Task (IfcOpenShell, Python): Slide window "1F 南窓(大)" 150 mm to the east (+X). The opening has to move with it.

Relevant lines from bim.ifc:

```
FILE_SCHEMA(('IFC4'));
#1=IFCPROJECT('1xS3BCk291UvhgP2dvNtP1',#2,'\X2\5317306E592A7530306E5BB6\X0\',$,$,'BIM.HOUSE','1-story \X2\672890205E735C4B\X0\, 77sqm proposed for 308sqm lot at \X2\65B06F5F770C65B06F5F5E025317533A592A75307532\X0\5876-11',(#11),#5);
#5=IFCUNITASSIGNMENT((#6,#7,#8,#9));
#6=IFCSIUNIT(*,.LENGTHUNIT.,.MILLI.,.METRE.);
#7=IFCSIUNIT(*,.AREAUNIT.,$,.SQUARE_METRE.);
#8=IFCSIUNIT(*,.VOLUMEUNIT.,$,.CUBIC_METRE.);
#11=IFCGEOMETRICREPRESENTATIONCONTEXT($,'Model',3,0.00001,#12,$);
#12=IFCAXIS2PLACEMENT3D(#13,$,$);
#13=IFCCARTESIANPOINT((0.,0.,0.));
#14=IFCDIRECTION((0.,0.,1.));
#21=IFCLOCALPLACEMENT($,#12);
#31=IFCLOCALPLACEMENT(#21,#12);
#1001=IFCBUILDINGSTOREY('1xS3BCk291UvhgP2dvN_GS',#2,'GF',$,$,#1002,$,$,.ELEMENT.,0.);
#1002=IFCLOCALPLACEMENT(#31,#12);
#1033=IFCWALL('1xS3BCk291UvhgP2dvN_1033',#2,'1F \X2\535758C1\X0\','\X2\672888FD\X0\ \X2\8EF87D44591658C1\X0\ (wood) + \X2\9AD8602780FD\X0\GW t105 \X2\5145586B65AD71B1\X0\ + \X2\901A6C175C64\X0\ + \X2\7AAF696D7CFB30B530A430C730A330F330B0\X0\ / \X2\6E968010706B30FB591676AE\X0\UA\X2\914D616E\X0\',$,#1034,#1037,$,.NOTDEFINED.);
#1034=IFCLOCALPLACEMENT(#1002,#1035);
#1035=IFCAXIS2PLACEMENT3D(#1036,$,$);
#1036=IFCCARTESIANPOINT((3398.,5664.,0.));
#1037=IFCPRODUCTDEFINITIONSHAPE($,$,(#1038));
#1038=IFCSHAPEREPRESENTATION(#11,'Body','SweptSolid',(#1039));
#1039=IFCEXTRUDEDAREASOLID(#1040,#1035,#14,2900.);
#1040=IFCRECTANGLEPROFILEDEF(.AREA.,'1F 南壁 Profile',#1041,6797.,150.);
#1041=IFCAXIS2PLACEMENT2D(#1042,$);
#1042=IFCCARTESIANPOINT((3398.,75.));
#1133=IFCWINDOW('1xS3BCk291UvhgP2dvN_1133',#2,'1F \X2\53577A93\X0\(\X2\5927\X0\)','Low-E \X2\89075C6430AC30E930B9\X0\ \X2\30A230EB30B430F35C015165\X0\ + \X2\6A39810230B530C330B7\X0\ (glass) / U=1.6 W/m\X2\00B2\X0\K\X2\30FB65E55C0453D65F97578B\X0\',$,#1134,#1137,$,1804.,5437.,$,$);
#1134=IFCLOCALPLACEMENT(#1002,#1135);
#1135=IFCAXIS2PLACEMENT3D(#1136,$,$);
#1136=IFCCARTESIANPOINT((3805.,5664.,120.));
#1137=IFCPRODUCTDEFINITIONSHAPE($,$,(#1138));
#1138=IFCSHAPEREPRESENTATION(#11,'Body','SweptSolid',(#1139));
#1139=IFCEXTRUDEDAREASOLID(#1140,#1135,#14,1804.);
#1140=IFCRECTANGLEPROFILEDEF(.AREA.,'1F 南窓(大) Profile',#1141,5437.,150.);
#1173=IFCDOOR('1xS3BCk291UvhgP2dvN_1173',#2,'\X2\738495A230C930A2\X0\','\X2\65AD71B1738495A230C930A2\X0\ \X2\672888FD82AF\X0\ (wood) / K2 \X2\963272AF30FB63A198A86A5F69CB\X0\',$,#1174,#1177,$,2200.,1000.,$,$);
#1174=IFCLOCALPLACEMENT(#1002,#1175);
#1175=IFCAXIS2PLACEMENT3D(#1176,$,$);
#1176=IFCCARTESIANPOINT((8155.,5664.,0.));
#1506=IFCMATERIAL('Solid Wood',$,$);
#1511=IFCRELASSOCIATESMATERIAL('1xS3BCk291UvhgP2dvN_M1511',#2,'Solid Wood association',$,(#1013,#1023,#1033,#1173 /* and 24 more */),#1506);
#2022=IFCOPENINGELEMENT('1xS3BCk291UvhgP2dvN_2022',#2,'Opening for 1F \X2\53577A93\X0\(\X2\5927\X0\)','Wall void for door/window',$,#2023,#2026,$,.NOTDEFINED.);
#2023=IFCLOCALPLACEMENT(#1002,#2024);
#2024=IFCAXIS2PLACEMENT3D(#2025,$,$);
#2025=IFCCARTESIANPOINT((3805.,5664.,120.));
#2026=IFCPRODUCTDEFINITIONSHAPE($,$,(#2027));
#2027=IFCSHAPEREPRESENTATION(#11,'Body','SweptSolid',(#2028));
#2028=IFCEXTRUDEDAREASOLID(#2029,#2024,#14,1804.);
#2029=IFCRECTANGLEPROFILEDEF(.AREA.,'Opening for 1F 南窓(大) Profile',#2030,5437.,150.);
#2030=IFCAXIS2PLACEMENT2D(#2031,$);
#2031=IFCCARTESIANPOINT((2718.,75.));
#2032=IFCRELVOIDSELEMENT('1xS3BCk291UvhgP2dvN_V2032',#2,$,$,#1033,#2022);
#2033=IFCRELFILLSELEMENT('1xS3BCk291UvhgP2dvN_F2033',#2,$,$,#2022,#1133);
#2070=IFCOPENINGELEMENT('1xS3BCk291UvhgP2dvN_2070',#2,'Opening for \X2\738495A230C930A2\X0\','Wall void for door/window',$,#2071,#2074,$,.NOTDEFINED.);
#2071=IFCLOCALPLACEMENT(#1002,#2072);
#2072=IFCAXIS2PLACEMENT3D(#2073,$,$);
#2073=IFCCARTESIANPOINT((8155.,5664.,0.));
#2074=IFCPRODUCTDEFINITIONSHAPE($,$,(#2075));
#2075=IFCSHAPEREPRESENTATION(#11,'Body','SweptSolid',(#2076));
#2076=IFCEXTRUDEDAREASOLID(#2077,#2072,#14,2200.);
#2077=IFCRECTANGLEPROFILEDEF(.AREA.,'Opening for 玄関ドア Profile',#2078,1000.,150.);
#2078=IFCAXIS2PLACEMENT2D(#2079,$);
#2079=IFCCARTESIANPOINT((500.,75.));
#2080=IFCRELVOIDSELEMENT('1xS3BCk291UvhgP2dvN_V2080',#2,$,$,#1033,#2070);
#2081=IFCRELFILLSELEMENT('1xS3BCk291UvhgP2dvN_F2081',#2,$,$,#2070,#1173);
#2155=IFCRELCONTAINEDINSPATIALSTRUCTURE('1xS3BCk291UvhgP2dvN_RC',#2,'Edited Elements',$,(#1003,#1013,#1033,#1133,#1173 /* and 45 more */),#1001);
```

```python
import ifcopenshell
import ifcopenshell.api.geometry
import ifcopenshell.util.placement

model = ifcopenshell.open("bim.ifc")

window = model.by_guid("1xS3BCk291UvhgP2dvN_1133")
opening = window.FillsVoids[0].RelatingOpeningElement
wall = opening.VoidsElements[0].RelatingBuildingElement

wall_matrix = ifcopenshell.util.placement.get_local_placement(wall.ObjectPlacement)
shift = wall_matrix[:3, 0] * 150.0
before = ifcopenshell.util.placement.get_local_placement(window.ObjectPlacement)[:3, 3].copy()

# The window is not placed relative to its opening, so move both.
for product in (opening, window):
    matrix = ifcopenshell.util.placement.get_local_placement(product.ObjectPlacement)
    matrix[:3, 3] += shift
    ifcopenshell.api.geometry.edit_object_placement(model, product=product, matrix=matrix, is_si=False)

after = ifcopenshell.util.placement.get_local_placement(window.ObjectPlacement)[:3, 3]
print("window moved by", (after - before).round(3) + 0.0)

model.write("bim_edited.ifc")
```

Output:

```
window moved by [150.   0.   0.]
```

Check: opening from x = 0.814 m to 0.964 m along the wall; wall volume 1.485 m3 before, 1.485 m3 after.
